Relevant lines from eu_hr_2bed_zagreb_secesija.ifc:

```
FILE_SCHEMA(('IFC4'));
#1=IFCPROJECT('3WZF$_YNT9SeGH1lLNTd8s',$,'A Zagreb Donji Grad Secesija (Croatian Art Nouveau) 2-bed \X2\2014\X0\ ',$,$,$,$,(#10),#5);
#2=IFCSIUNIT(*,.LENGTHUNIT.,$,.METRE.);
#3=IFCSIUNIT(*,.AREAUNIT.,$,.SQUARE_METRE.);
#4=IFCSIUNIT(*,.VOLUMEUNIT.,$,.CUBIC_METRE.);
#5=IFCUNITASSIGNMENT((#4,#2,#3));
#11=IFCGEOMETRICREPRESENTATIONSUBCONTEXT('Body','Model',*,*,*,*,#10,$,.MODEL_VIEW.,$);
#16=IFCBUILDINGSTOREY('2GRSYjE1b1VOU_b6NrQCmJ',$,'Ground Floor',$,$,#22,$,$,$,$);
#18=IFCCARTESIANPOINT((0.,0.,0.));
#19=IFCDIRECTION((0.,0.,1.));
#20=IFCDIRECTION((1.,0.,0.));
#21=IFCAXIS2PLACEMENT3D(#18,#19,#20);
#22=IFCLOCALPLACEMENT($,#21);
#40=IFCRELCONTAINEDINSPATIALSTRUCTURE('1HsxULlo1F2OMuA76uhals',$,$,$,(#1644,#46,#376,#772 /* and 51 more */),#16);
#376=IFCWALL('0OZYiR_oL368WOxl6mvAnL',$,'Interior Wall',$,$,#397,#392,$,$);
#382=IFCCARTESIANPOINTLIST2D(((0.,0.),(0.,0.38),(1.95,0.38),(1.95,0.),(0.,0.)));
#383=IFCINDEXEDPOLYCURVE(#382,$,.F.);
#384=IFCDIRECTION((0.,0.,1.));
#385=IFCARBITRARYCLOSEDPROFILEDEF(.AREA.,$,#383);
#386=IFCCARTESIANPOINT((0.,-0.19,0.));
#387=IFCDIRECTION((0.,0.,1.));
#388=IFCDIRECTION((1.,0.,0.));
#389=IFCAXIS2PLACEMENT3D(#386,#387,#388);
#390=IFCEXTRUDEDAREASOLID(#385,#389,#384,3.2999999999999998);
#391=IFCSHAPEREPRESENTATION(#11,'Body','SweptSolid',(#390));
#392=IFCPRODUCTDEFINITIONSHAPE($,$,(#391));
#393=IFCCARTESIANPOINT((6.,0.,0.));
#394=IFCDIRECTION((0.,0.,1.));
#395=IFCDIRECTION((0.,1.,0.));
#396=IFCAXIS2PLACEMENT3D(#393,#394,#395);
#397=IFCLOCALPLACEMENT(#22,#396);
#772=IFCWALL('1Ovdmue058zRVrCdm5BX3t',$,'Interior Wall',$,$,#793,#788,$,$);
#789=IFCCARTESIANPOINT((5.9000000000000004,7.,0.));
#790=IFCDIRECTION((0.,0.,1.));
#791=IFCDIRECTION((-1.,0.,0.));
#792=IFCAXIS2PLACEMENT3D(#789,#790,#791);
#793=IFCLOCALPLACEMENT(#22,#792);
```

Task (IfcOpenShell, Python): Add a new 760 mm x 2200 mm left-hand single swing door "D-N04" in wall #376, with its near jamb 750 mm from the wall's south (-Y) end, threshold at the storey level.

```python
import numpy as np
import ifcopenshell
import ifcopenshell.api.feature
import ifcopenshell.api.geometry
import ifcopenshell.api.root
import ifcopenshell.api.spatial
import ifcopenshell.geom
import ifcopenshell.util.element
import ifcopenshell.util.placement
import ifcopenshell.util.representation
import ifcopenshell.util.shape
import ifcopenshell.util.unit

model = ifcopenshell.open("eu_hr_2bed_zagreb_secesija.ifc")
unit_scale = ifcopenshell.util.unit.calculate_unit_scale(model)
settings = ifcopenshell.geom.settings()


def volume(element):
    """Net volume in cubic metres, openings subtracted."""
    shape = ifcopenshell.geom.create_shape(settings, element)
    return ifcopenshell.util.shape.get_volume(shape.geometry)


wall = model.by_guid("0OZYiR_oL368WOxl6mvAnL")
storey = ifcopenshell.util.element.get_container(wall, ifc_class="IfcBuildingStorey")
context = ifcopenshell.util.representation.get_context(model, "Model", "Body", "MODEL_VIEW")
before = volume(wall)

width, height, from_end, sill = 0.76, 2.2, 0.75, 0.0  # metres

# The wall runs along its own X axis, and the end named is its -X end.
wall_shape = ifcopenshell.geom.create_shape(settings, wall)
x, y, z = ifcopenshell.util.shape.get_vertices(wall_shape.geometry).T
start = x.min() + from_end
face, thickness = float(y.min()), float(y.max() - y.min())
wall_matrix = ifcopenshell.util.placement.get_local_placement(wall.ObjectPlacement)
level = ifcopenshell.util.placement.get_local_placement(storey.ObjectPlacement)[2, 3]


def in_wall(x, y):
    """Placement at x, y metres in the wall's axes, at sill height."""
    matrix = wall_matrix.copy()
    matrix[:, 3] = wall_matrix @ np.array([x / unit_scale, y / unit_scale, 0.0, 1.0])
    matrix[2, 3] = level + sill / unit_scale
    return matrix


# Opening: a box that overshoots both wall faces by 50 mm.
opening = ifcopenshell.api.root.create_entity(model, ifc_class="IfcOpeningElement", predefined_type="OPENING")
box = ifcopenshell.api.geometry.add_wall_representation(
    model, context=context, length=width, height=height, thickness=thickness + 0.1
)
ifcopenshell.api.geometry.assign_representation(model, product=opening, representation=box)
ifcopenshell.api.geometry.edit_object_placement(model, product=opening, matrix=in_wall(start, face - 0.05), is_si=False)
ifcopenshell.api.feature.add_feature(model, feature=opening, element=wall)

door = ifcopenshell.api.root.create_entity(model, ifc_class="IfcDoor", name="D-N04", predefined_type="DOOR")
door.OverallWidth, door.OverallHeight = width / unit_scale, height / unit_scale
door.OperationType = "SINGLE_SWING_LEFT"
body = ifcopenshell.api.geometry.add_door_representation(
    model,
    context=context,
    overall_width=door.OverallWidth,
    overall_height=door.OverallHeight,
    operation_type="SINGLE_SWING_LEFT",
    lining_properties={"LiningDepth": thickness / unit_scale, "ThresholdDepth": thickness / unit_scale},
)
ifcopenshell.api.geometry.assign_representation(model, product=door, representation=body)
ifcopenshell.api.spatial.assign_container(model, products=[door], relating_structure=storey)
ifcopenshell.api.feature.add_filling(model, opening=opening, element=door)

# The lining spans the wall, so the door starts at the wall face.
ifcopenshell.api.geometry.edit_object_placement(model, product=door, matrix=in_wall(start, face), is_si=False)

after = volume(wall)

print(f"wall volume {before:.3f} -> {after:.3f} m3")

model.write("eu_hr_2bed_zagreb_secesija_updated.ifc")
```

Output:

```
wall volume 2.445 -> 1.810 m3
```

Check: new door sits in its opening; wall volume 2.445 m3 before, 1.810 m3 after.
